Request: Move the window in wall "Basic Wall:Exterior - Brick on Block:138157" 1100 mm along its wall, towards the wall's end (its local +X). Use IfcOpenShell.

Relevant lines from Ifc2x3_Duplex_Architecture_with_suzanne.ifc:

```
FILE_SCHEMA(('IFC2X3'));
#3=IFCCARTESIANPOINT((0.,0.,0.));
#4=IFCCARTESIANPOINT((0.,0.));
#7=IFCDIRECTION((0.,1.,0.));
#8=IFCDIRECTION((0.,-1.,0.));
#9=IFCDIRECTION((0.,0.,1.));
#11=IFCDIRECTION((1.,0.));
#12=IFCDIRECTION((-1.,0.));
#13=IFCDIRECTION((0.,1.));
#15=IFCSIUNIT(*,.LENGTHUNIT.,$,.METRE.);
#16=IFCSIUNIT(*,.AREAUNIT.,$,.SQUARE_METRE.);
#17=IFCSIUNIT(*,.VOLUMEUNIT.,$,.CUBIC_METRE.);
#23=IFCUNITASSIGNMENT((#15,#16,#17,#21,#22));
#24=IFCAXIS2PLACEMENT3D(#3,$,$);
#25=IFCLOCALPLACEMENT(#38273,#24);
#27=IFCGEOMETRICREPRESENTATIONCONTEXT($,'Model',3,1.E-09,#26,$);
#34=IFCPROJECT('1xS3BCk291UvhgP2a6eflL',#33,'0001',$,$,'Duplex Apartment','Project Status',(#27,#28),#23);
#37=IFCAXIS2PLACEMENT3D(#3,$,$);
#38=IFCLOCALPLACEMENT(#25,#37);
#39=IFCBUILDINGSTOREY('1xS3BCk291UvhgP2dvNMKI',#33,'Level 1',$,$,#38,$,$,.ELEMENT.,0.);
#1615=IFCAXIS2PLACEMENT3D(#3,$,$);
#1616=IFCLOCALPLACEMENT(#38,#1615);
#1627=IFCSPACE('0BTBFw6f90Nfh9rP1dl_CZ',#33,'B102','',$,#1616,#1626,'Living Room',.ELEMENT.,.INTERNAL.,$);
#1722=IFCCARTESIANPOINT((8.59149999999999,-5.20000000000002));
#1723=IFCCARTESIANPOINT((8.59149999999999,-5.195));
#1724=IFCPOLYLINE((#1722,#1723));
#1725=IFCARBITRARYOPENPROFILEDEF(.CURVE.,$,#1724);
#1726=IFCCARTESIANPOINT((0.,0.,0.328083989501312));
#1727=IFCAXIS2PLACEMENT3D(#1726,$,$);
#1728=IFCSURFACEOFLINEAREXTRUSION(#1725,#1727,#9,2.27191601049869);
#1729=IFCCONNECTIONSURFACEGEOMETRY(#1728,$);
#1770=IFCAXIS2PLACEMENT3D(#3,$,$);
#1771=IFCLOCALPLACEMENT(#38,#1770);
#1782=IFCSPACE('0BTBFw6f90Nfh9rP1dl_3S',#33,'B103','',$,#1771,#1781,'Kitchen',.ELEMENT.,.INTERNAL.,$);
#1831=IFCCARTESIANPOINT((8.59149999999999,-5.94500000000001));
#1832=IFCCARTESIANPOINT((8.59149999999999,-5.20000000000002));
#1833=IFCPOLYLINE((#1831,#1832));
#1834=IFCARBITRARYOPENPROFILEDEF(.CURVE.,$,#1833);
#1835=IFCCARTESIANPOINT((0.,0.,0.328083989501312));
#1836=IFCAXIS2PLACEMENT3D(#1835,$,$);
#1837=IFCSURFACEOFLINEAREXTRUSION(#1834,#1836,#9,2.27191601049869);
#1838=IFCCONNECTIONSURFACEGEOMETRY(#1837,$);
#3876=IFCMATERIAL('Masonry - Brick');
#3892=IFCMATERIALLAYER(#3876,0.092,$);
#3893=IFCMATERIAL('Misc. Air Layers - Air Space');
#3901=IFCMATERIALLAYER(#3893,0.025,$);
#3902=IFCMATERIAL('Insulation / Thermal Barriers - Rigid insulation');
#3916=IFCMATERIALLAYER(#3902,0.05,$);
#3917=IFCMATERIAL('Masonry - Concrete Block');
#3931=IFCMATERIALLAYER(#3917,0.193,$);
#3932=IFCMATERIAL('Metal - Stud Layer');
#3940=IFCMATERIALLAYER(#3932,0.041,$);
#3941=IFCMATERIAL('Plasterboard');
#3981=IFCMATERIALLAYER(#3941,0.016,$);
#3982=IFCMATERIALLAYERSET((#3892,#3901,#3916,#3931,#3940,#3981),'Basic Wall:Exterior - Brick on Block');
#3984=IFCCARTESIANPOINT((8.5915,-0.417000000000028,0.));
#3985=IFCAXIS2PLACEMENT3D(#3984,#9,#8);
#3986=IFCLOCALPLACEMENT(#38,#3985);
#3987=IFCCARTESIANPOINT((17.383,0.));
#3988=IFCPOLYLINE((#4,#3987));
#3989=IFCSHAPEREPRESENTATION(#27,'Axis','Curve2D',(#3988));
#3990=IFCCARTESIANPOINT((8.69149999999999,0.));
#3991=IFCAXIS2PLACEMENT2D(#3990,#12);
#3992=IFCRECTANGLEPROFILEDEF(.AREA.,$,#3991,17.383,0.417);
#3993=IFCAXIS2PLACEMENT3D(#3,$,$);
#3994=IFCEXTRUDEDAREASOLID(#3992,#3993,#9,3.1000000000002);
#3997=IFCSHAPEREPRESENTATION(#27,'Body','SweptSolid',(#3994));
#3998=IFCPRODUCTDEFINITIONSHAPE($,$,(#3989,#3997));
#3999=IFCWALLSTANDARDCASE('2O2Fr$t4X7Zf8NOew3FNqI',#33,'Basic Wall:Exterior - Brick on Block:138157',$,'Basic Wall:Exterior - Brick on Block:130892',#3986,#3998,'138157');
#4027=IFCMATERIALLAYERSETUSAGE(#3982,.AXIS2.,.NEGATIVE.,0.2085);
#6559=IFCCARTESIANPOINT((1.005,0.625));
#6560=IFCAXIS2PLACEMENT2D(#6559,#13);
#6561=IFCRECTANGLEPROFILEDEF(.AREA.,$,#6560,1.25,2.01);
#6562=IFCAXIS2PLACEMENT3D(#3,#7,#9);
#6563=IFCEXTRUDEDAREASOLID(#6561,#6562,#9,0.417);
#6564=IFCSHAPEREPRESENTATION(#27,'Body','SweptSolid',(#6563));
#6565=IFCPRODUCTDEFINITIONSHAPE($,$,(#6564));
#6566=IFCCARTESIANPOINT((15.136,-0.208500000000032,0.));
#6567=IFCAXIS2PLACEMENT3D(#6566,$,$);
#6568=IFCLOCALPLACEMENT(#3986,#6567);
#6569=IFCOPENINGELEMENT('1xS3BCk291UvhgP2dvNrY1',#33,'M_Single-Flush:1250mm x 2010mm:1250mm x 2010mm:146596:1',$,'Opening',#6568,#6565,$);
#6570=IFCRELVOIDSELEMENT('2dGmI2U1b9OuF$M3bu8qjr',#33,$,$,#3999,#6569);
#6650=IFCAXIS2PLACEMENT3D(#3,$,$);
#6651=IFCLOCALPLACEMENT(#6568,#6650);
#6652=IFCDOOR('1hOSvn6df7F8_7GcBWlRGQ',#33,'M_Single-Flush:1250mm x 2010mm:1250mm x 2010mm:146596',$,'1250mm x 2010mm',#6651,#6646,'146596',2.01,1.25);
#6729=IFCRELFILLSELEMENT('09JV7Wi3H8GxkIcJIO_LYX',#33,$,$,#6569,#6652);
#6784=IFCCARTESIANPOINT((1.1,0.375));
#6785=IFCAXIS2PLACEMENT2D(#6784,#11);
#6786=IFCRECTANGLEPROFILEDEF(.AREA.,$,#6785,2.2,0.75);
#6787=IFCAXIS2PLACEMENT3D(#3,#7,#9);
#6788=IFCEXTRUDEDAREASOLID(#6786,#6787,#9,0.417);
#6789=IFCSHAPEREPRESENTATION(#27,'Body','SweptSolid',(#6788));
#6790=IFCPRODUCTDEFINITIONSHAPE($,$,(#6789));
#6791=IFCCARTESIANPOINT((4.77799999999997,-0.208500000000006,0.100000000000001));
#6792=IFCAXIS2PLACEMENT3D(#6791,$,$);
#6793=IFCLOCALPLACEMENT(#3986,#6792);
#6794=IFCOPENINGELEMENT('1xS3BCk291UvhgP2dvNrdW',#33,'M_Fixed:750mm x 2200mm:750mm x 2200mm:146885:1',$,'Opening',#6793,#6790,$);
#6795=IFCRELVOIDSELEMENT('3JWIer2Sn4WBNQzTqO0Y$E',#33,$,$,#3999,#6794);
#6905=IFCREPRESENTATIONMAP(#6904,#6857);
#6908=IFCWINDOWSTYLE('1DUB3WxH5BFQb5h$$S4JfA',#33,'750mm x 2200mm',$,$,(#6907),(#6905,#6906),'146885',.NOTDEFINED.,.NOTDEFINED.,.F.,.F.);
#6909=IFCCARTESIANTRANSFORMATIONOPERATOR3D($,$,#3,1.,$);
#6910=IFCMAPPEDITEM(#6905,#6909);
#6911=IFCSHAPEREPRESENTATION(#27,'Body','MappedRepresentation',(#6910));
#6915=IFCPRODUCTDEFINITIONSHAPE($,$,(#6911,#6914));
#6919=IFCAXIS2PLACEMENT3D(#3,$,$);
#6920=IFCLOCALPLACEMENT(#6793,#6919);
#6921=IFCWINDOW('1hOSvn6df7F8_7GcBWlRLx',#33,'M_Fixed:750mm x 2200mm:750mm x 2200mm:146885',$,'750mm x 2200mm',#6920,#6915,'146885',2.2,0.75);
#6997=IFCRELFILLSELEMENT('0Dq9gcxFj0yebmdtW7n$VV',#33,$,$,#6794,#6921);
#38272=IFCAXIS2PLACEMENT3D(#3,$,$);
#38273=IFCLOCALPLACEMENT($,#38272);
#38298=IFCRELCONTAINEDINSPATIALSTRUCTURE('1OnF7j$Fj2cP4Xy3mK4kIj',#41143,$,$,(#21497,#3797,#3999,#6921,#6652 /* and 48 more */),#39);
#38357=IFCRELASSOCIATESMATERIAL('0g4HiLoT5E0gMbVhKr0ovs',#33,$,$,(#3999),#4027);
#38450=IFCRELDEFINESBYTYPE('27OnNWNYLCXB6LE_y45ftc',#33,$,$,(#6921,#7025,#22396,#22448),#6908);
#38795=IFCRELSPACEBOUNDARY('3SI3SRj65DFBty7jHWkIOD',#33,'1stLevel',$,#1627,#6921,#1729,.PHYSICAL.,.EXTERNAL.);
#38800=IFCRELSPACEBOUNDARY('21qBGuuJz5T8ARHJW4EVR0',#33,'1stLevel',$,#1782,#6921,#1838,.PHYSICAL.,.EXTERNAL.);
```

```python
import numpy as np
import ifcopenshell
import ifcopenshell.api.geometry
import ifcopenshell.util.placement
import ifcopenshell.util.unit

model = ifcopenshell.open("Ifc2x3_Duplex_Architecture_with_suzanne.ifc")
unit_scale = ifcopenshell.util.unit.calculate_unit_scale(model)

window = model.by_guid("1hOSvn6df7F8_7GcBWlRLx")
opening = window.FillsVoids[0].RelatingOpeningElement
wall = opening.VoidsElements[0].RelatingBuildingElement

wall_matrix = ifcopenshell.util.placement.get_local_placement(wall.ObjectPlacement)
shift = wall_matrix[:3, 0] * 1.1 / unit_scale
before = ifcopenshell.util.placement.get_local_placement(window.ObjectPlacement)[:3, 3].copy()

# The window is placed relative to its opening, so it follows when the opening moves.
matrix = ifcopenshell.util.placement.get_local_placement(opening.ObjectPlacement)
matrix[:3, 3] += shift
ifcopenshell.api.geometry.edit_object_placement(
    model, product=opening, matrix=matrix, is_si=False, should_transform_children=True
)

# Space boundary surfaces are stored in each space's coordinates; move them too.
for rel in window.ProvidesBoundaries:
    if not rel.ConnectionGeometry:
        continue
    surface = rel.ConnectionGeometry.SurfaceOnRelatingElement
    space_matrix = ifcopenshell.util.placement.get_local_placement(rel.RelatingSpace.ObjectPlacement)
    point = np.array(surface.Position.Location.Coordinates) + space_matrix[:3, :3].T @ shift
    surface.Position = model.createIfcAxis2Placement3D(
        model.createIfcCartesianPoint(point.tolist()), surface.Position.Axis, surface.Position.RefDirection
    )

after = ifcopenshell.util.placement.get_local_placement(window.ObjectPlacement)[:3, 3]
print("window moved by", (after - before).round(3) + 0.0)

model.write("Ifc2x3_Duplex_Architecture_with_suzanne_v2.ifc")
```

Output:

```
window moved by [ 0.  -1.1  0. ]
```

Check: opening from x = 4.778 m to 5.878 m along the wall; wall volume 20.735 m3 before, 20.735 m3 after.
